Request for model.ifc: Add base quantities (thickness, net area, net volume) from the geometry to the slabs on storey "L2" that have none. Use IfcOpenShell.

First a look at what the model holds.

```python
import ifcopenshell
import ifcopenshell.util.element
import ifcopenshell.util.unit

model = ifcopenshell.open("model.ifc")
print(model.schema)
for unit_type in ("LENGTHUNIT", "AREAUNIT", "VOLUMEUNIT"):
    print(unit_type, ifcopenshell.util.unit.calculate_unit_scale(model, unit_type))
storey = next(s for s in model.by_type("IfcBuildingStorey") if s.Name == "L2")
slabs = [e for e in ifcopenshell.util.element.get_decomposition(storey) if e.is_a("IfcSlab")]
for e in sorted(slabs, key=lambda e: e.id()):
    print(e.id(), e.is_a(), e.Name, list(ifcopenshell.util.element.get_psets(e, qtos_only=True)), sep=" | ")
```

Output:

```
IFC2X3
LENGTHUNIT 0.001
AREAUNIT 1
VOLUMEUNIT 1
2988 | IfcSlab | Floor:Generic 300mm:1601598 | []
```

```python
import ifcopenshell
import ifcopenshell.api.pset
import ifcopenshell.geom
import ifcopenshell.util.element
import ifcopenshell.util.shape
import ifcopenshell.util.unit

model = ifcopenshell.open("model.ifc")
unit_scale = ifcopenshell.util.unit.calculate_unit_scale(model)
area_scale = ifcopenshell.util.unit.calculate_unit_scale(model, "AREAUNIT")
volume_scale = ifcopenshell.util.unit.calculate_unit_scale(model, "VOLUMEUNIT")
settings = ifcopenshell.geom.settings()

storey = next(s for s in model.by_type("IfcBuildingStorey") if s.Name == "L2")
slabs = [e for e in ifcopenshell.util.element.get_decomposition(storey) if e.is_a("IfcSlab")]

for e in sorted(slabs, key=lambda e: e.id()):
    if ifcopenshell.util.element.get_psets(e, qtos_only=True, should_inherit=False):
        continue
    # Geometry comes back in metres, in the element's own axes.
    shape = ifcopenshell.geom.create_shape(settings, e)
    values = {
        "Width": ifcopenshell.util.shape.get_z(shape.geometry) / unit_scale,
        "NetArea": ifcopenshell.util.shape.get_footprint_area(shape.geometry) / area_scale,
        "NetVolume": ifcopenshell.util.shape.get_volume(shape.geometry) / volume_scale,
    }
    qto = ifcopenshell.api.pset.add_qto(model, product=e, name="BaseQuantities")
    ifcopenshell.api.pset.edit_qto(model, qto=qto, properties=values)
    print(e.id(), {k: round(v, 3) for k, v in values.items()})

model.write("model_v2.ifc")
```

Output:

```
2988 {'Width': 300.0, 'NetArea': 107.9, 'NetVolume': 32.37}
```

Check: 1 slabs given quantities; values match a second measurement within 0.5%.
